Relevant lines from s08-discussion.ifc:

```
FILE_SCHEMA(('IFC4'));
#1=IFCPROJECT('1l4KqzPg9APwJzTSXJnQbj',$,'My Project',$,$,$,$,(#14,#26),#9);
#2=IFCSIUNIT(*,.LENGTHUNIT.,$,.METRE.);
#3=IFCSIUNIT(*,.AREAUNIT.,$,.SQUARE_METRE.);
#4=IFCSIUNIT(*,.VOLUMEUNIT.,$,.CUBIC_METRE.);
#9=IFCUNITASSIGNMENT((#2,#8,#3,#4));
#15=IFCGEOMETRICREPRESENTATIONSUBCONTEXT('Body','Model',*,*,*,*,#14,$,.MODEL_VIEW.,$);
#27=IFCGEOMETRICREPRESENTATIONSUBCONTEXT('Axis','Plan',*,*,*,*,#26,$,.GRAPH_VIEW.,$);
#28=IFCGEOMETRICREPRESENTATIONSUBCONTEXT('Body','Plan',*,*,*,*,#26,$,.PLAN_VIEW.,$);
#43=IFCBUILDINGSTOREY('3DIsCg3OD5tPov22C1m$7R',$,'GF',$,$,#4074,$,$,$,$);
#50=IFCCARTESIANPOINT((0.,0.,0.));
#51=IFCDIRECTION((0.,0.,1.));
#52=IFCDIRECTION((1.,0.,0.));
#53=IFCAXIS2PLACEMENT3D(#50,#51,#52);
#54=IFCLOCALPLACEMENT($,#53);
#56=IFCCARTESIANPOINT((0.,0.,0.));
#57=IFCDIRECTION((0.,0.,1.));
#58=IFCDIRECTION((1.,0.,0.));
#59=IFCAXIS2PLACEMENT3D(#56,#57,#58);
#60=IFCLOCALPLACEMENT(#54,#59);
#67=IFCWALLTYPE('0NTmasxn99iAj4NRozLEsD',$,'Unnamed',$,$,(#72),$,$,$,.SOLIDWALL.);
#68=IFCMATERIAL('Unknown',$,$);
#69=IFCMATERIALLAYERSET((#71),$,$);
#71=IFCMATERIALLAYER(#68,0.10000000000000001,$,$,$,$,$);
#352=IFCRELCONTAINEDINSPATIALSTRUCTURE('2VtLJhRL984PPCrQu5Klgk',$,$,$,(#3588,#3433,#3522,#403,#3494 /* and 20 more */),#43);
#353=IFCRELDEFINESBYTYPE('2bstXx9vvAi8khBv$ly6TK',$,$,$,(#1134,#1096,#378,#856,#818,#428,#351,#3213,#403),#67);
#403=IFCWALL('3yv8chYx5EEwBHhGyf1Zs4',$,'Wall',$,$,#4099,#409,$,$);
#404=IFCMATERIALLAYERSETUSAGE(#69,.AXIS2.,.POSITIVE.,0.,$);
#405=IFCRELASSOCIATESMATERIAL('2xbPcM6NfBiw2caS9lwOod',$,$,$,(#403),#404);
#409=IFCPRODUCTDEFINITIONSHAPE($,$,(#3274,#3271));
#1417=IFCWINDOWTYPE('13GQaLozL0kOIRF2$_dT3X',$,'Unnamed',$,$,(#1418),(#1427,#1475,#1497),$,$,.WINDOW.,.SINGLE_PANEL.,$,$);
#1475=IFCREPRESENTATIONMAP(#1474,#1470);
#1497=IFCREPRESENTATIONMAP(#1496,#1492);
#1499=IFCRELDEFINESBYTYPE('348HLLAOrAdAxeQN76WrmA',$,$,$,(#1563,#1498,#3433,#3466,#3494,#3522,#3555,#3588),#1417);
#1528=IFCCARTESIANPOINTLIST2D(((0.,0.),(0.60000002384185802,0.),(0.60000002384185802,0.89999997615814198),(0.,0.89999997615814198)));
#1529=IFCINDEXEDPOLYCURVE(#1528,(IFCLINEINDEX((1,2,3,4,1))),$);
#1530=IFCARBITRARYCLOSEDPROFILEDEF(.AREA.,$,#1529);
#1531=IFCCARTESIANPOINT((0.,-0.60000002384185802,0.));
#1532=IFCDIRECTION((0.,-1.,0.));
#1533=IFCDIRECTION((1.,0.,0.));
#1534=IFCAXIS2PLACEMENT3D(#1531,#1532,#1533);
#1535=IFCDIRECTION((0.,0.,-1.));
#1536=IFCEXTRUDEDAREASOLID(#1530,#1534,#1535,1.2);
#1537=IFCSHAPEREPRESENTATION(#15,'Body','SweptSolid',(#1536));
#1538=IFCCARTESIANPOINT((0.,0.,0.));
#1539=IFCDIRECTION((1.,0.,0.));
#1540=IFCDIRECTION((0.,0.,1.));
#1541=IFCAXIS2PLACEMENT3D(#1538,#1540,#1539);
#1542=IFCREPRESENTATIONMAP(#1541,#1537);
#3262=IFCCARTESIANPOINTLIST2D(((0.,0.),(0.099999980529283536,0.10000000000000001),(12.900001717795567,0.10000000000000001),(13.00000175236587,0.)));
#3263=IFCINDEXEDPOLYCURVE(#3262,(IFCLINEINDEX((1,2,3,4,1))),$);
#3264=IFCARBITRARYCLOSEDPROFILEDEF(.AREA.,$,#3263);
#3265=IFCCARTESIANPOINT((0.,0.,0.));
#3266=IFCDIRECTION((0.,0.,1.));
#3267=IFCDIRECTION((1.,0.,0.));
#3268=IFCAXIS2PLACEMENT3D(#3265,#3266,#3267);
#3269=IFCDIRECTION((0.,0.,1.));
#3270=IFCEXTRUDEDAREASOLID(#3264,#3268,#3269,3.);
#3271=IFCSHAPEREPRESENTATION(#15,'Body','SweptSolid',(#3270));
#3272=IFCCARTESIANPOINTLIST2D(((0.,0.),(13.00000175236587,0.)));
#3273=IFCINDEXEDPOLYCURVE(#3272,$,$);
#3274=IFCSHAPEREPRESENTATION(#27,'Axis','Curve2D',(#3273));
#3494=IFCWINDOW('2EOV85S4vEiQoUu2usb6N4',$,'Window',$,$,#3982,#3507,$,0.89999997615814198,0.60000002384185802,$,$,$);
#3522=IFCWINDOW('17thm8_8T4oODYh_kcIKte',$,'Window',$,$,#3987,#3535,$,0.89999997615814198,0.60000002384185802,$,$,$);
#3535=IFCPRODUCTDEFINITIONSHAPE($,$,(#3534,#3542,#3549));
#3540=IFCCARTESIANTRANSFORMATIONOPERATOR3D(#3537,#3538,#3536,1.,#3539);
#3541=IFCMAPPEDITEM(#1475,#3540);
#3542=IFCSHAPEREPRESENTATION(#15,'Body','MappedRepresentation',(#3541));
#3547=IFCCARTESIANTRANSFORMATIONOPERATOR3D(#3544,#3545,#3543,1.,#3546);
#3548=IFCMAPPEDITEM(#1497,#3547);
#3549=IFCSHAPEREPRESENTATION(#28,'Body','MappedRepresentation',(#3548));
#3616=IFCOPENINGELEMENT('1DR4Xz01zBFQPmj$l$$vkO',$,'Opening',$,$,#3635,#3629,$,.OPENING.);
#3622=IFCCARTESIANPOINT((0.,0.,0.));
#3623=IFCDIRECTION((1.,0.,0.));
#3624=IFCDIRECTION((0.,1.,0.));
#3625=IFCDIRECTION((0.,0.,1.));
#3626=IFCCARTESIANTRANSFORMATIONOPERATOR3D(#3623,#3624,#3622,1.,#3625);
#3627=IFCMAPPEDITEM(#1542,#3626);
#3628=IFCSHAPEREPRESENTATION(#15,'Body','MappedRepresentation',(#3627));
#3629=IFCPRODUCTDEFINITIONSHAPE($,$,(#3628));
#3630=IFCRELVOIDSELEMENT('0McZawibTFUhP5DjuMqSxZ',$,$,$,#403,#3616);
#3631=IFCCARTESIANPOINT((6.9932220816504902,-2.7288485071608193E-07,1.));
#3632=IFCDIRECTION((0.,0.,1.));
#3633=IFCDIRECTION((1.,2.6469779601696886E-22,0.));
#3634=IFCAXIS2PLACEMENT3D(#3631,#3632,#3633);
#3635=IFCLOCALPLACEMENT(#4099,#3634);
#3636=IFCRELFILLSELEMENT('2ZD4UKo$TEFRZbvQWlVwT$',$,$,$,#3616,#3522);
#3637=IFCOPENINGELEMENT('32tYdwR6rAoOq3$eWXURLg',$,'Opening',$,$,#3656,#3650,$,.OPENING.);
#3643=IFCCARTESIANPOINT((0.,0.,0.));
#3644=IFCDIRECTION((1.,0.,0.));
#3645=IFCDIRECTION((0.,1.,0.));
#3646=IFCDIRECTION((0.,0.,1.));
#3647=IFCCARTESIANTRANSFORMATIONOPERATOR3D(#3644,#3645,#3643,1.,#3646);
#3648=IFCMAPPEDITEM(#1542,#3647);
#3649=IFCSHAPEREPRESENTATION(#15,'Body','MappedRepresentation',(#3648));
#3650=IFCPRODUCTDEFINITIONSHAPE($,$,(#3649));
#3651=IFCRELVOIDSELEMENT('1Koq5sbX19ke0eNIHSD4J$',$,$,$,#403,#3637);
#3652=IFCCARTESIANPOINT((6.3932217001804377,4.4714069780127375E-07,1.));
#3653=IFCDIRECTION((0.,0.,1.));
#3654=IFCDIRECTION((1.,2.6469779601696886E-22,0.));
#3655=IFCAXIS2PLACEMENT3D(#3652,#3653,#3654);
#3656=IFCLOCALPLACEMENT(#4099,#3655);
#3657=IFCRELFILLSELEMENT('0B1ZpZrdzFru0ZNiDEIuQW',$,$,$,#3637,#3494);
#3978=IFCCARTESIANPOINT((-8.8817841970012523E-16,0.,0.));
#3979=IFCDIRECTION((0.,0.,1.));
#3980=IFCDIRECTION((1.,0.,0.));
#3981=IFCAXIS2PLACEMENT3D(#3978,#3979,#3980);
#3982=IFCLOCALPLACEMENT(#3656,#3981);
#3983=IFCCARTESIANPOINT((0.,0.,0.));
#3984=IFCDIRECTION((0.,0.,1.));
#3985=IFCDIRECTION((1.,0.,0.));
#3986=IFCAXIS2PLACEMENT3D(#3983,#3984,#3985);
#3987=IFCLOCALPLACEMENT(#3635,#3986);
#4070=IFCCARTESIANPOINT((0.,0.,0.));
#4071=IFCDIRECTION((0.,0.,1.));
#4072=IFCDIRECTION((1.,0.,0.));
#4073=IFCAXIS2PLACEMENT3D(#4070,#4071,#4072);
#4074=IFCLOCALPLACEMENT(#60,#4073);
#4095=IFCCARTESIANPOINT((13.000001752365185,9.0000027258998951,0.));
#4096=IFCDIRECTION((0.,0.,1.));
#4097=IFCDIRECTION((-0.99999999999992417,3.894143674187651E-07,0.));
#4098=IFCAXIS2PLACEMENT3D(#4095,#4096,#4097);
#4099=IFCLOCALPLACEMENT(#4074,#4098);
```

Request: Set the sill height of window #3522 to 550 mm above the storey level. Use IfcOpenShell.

```python
import numpy as np
import ifcopenshell
import ifcopenshell.api.geometry
import ifcopenshell.geom
import ifcopenshell.util.element
import ifcopenshell.util.placement
import ifcopenshell.util.shape
import ifcopenshell.util.unit

model = ifcopenshell.open("s08-discussion.ifc")
unit_scale = ifcopenshell.util.unit.calculate_unit_scale(model)

window = model.by_guid("17thm8_8T4oODYh_kcIKte")
opening = window.FillsVoids[0].RelatingOpeningElement
storey = ifcopenshell.util.element.get_container(window, ifc_class="IfcBuildingStorey")
level = ifcopenshell.util.placement.get_local_placement(storey.ObjectPlacement)[2, 3]

# The opening's origin need not be at the sill, so measure its lowest point.
shape = ifcopenshell.geom.create_shape(ifcopenshell.geom.settings(), opening)
bottom = ifcopenshell.util.shape.get_shape_bottom_elevation(shape, shape.geometry) / unit_scale
dz = level + 0.55 / unit_scale - bottom

shift = np.array([0.0, 0.0, dz])
# The window is placed relative to its opening, so it follows when the opening moves.
matrix = ifcopenshell.util.placement.get_local_placement(opening.ObjectPlacement)
matrix[:3, 3] += shift
ifcopenshell.api.geometry.edit_object_placement(
    model, product=opening, matrix=matrix, is_si=False, should_transform_children=True
)

print(f"moved by {dz * unit_scale:+.3f} m")

model.write("s08-discussion-out.ifc")
```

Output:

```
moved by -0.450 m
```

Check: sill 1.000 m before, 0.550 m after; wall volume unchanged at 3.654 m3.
